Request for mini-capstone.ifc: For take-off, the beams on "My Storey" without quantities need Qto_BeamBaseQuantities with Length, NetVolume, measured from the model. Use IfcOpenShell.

First a look at what the model holds.

```python
import ifcopenshell
import ifcopenshell.util.element
import ifcopenshell.util.unit

model = ifcopenshell.open("mini-capstone.ifc")
print(model.schema)
for unit_type in ("LENGTHUNIT", "AREAUNIT", "VOLUMEUNIT"):
    print(unit_type, ifcopenshell.util.unit.calculate_unit_scale(model, unit_type))
storey = next(s for s in model.by_type("IfcBuildingStorey") if s.Name == "My Storey")
beams = [e for e in ifcopenshell.util.element.get_decomposition(storey) if e.is_a("IfcBeam")]
for e in sorted(beams, key=lambda e: e.id()):
    print(e.id(), e.is_a(), e.Name, list(ifcopenshell.util.element.get_psets(e, qtos_only=True)), sep=" | ")
```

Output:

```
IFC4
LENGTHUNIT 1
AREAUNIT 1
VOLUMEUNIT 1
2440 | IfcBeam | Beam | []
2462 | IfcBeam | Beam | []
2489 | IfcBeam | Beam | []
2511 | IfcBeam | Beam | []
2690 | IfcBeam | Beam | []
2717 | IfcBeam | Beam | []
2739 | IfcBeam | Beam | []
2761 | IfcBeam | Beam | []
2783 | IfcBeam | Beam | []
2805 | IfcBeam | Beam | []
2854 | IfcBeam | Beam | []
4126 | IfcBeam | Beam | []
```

```python
import ifcopenshell
import ifcopenshell.api.pset
import ifcopenshell.geom
import ifcopenshell.util.element
import ifcopenshell.util.shape
import ifcopenshell.util.unit

model = ifcopenshell.open("mini-capstone.ifc")
unit_scale = ifcopenshell.util.unit.calculate_unit_scale(model)
volume_scale = ifcopenshell.util.unit.calculate_unit_scale(model, "VOLUMEUNIT")
settings = ifcopenshell.geom.settings()

storey = next(s for s in model.by_type("IfcBuildingStorey") if s.Name == "My Storey")
beams = [e for e in ifcopenshell.util.element.get_decomposition(storey) if e.is_a("IfcBeam")]

for e in sorted(beams, key=lambda e: e.id()):
    if ifcopenshell.util.element.get_psets(e, qtos_only=True, should_inherit=False):
        continue
    # Geometry comes back in metres, in the element's own axes.
    shape = ifcopenshell.geom.create_shape(settings, e)
    values = {
        "Length": ifcopenshell.util.shape.get_max_xyz(shape.geometry) / unit_scale,
        "NetVolume": ifcopenshell.util.shape.get_volume(shape.geometry) / volume_scale,
    }
    qto = ifcopenshell.api.pset.add_qto(model, product=e, name="Qto_BeamBaseQuantities")
    ifcopenshell.api.pset.edit_qto(model, qto=qto, properties=values)
    print(e.id(), {k: round(v, 3) for k, v in values.items()})

model.write("mini-capstone-out.ifc")
```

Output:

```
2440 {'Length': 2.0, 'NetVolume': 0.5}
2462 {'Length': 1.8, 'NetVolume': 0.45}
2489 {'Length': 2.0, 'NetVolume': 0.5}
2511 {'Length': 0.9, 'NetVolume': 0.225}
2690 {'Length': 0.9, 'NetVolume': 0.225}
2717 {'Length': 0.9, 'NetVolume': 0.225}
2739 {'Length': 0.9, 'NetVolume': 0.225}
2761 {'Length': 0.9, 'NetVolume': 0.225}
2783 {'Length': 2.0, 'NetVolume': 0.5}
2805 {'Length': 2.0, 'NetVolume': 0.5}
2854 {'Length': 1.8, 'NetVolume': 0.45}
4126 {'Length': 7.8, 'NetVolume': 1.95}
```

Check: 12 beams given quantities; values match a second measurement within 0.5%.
